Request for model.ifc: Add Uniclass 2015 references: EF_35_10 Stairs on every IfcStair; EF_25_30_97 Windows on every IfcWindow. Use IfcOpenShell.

First a look at what the model holds.

```python
import ifcopenshell

model = ifcopenshell.open("model.ifc")
print(model.schema)
print("classifications:", [c.Name for c in model.by_type("IfcClassification")])
for ifc_class in ("IfcDoor", "IfcRoof", "IfcStair", "IfcWall", "IfcWindow"):
    print(ifc_class, len(model.by_type(ifc_class)))
```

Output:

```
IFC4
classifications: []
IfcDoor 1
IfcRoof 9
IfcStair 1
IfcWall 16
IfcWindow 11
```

```python
import ifcopenshell
import ifcopenshell.api.classification

model = ifcopenshell.open("model.ifc")

system = ifcopenshell.api.classification.add_classification(model, classification="Uniclass 2015")

codes = {
    "IfcStair": ("EF_35_10", "Stairs"),
    "IfcWindow": ("EF_25_30_97", "Windows"),
}
for ifc_class, (code, name) in codes.items():
    products = model.by_type(ifc_class)
    ifcopenshell.api.classification.add_reference(
        model, products=products, classification=system, identification=code, name=name
    )
    print(code, len(products))

model.write("model_rev.ifc")
```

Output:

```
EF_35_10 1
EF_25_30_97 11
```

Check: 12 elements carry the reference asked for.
